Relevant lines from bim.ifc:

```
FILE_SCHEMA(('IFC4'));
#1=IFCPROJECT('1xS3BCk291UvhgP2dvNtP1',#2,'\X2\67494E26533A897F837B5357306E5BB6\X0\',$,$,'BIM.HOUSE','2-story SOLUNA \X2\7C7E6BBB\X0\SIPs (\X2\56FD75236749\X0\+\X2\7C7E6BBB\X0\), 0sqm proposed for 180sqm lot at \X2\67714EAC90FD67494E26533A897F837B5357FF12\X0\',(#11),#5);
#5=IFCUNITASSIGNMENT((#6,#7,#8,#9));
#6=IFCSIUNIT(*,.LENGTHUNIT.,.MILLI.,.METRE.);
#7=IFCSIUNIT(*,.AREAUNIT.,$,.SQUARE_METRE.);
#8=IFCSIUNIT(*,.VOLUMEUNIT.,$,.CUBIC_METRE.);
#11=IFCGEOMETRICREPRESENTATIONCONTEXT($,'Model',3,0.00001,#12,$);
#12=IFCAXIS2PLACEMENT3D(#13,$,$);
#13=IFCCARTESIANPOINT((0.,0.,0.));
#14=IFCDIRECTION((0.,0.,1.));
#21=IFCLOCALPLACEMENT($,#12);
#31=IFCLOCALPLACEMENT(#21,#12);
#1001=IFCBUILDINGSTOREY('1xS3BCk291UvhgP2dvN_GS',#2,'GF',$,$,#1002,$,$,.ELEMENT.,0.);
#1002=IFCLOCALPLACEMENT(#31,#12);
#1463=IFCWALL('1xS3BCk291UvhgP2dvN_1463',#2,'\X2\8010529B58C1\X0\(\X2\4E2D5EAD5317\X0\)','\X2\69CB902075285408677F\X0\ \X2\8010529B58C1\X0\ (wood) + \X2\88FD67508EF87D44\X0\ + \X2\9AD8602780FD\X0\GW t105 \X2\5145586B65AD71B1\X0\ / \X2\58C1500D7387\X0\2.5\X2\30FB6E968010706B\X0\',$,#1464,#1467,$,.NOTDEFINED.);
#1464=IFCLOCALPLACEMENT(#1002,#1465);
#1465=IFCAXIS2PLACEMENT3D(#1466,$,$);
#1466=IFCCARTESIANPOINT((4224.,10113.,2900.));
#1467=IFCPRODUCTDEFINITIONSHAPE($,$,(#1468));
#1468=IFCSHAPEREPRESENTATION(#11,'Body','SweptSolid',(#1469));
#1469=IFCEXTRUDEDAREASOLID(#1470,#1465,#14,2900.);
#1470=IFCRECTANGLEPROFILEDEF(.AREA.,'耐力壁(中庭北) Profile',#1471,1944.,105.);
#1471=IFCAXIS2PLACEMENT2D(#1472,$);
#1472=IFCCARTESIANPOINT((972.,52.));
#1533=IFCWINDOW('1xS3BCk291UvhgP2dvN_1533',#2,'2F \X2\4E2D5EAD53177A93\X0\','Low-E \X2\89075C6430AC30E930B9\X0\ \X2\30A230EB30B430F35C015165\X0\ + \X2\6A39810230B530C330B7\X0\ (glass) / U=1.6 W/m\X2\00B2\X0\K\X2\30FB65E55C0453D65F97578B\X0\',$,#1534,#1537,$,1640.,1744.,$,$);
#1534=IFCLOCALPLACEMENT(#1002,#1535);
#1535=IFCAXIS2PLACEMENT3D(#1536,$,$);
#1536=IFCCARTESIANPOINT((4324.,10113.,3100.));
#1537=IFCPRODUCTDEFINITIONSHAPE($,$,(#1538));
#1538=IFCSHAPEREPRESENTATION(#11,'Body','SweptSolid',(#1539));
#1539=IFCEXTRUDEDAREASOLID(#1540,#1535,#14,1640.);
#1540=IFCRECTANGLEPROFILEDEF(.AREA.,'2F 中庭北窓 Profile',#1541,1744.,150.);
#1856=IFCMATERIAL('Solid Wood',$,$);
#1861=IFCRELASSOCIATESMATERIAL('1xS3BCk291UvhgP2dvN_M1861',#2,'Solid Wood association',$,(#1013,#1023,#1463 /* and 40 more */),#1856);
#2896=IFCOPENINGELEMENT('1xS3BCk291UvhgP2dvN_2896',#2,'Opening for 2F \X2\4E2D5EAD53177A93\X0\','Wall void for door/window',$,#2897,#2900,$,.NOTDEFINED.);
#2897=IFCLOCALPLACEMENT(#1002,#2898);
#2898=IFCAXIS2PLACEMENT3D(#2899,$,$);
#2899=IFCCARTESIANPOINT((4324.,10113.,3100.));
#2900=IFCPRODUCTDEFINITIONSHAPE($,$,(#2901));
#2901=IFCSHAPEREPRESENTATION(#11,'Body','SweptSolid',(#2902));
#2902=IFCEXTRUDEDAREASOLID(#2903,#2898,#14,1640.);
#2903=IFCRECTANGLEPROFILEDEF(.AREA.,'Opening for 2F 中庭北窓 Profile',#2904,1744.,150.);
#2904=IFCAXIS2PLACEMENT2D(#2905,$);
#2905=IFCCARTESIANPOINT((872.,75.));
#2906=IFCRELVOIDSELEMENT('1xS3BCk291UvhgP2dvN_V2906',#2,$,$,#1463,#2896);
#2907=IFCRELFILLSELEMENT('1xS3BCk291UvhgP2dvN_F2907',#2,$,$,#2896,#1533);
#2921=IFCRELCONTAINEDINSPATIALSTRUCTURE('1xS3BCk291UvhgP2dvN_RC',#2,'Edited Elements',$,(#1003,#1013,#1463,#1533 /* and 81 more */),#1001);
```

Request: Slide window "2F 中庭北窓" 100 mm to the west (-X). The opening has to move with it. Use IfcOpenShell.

```python
import ifcopenshell
import ifcopenshell.api.geometry
import ifcopenshell.util.placement
import ifcopenshell.util.unit

model = ifcopenshell.open("bim.ifc")
unit_scale = ifcopenshell.util.unit.calculate_unit_scale(model)

window = model.by_guid("1xS3BCk291UvhgP2dvN_1533")
opening = window.FillsVoids[0].RelatingOpeningElement
wall = opening.VoidsElements[0].RelatingBuildingElement

wall_matrix = ifcopenshell.util.placement.get_local_placement(wall.ObjectPlacement)
shift = wall_matrix[:3, 0] * -0.1 / unit_scale
before = ifcopenshell.util.placement.get_local_placement(window.ObjectPlacement)[:3, 3].copy()

# The window is not placed relative to its opening, so move both.
for product in (opening, window):
    matrix = ifcopenshell.util.placement.get_local_placement(product.ObjectPlacement)
    matrix[:3, 3] += shift
    ifcopenshell.api.geometry.edit_object_placement(model, product=product, matrix=matrix, is_si=False)

after = ifcopenshell.util.placement.get_local_placement(window.ObjectPlacement)[:3, 3]
print("window moved by", (after - before).round(3) + 0.0)

model.write("bim_v2.ifc")
```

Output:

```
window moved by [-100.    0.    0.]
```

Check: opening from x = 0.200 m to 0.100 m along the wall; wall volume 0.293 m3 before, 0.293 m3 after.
